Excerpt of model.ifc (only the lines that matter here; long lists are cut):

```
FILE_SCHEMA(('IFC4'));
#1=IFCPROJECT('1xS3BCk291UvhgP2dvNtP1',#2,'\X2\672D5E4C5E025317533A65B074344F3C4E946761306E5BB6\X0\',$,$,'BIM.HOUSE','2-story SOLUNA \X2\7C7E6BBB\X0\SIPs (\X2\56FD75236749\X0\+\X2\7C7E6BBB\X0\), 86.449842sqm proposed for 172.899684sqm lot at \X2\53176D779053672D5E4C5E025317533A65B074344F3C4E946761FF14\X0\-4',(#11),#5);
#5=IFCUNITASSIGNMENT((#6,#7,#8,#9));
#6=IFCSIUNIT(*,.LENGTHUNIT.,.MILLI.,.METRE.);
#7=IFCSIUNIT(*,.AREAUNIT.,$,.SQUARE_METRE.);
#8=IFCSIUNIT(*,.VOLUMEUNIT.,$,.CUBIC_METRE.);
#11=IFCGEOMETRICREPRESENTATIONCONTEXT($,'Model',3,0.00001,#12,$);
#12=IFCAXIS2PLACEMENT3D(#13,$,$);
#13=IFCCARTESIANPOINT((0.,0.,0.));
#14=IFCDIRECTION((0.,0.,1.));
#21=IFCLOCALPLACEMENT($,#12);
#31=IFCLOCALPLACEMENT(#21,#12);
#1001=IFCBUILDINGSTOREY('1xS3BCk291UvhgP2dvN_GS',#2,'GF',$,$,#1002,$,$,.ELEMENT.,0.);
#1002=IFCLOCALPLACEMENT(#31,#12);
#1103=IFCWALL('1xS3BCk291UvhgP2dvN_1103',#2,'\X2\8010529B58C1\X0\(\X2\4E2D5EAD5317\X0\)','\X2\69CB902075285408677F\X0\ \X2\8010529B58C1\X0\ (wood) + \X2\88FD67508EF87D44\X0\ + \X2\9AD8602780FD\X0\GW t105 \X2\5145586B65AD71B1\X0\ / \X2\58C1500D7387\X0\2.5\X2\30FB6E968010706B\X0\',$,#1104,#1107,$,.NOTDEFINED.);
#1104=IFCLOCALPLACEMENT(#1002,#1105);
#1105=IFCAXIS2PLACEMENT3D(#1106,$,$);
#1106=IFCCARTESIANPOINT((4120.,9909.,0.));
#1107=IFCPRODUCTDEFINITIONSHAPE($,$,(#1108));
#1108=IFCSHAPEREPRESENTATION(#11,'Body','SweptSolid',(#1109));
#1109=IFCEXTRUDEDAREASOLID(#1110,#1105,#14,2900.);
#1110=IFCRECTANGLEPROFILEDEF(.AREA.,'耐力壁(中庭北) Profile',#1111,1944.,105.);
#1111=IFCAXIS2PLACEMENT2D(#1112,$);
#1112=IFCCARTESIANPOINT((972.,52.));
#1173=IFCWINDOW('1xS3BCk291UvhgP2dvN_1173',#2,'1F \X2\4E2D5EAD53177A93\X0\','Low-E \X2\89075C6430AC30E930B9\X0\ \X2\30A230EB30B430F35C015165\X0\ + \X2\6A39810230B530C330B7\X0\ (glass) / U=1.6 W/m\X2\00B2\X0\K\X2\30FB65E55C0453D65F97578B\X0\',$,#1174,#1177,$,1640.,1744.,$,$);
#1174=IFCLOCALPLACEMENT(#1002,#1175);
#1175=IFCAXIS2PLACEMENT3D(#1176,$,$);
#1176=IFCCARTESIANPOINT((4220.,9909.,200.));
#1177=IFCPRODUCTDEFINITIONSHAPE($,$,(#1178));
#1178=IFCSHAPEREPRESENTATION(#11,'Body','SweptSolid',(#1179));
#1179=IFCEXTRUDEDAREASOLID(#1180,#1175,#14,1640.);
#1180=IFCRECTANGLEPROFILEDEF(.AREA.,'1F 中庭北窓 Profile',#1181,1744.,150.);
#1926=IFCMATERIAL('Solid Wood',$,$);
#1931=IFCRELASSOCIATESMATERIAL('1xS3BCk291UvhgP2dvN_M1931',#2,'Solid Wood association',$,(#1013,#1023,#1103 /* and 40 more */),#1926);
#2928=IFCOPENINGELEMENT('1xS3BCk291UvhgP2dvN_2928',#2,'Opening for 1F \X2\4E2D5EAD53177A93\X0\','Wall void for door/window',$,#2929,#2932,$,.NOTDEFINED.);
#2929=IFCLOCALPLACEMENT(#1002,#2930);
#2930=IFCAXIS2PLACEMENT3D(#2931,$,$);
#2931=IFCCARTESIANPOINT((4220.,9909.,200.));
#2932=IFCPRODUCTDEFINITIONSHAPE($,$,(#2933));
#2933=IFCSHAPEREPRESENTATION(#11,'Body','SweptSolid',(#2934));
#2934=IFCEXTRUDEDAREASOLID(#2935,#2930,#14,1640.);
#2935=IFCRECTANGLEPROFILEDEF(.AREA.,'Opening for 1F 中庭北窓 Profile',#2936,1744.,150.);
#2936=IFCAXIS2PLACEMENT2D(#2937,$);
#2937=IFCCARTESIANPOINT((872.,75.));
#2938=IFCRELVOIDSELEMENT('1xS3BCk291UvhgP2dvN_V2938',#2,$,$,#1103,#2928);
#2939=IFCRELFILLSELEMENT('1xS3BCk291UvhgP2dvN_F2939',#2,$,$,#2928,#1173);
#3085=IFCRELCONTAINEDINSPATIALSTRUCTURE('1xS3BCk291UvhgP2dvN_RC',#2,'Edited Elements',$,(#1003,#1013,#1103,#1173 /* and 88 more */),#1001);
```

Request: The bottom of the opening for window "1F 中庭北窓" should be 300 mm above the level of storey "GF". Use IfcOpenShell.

```python
import numpy as np
import ifcopenshell
import ifcopenshell.api.geometry
import ifcopenshell.geom
import ifcopenshell.util.element
import ifcopenshell.util.placement
import ifcopenshell.util.shape
import ifcopenshell.util.unit

model = ifcopenshell.open("model.ifc")
unit_scale = ifcopenshell.util.unit.calculate_unit_scale(model)

window = model.by_guid("1xS3BCk291UvhgP2dvN_1173")
opening = window.FillsVoids[0].RelatingOpeningElement
storey = ifcopenshell.util.element.get_container(window, ifc_class="IfcBuildingStorey")
level = ifcopenshell.util.placement.get_local_placement(storey.ObjectPlacement)[2, 3]

# The opening's origin need not be at the sill, so measure its lowest point.
shape = ifcopenshell.geom.create_shape(ifcopenshell.geom.settings(), opening)
bottom = ifcopenshell.util.shape.get_shape_bottom_elevation(shape, shape.geometry) / unit_scale
dz = level + 300.0 - bottom

shift = np.array([0.0, 0.0, dz])
# The window is not placed relative to its opening, so move both.
for product in (opening, window):
    matrix = ifcopenshell.util.placement.get_local_placement(product.ObjectPlacement)
    matrix[:3, 3] += shift
    ifcopenshell.api.geometry.edit_object_placement(model, product=product, matrix=matrix, is_si=False)

print(f"moved by {dz * unit_scale:+.3f} m")

model.write("model_rev.ifc")
```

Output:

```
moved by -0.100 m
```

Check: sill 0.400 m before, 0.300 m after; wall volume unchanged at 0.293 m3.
